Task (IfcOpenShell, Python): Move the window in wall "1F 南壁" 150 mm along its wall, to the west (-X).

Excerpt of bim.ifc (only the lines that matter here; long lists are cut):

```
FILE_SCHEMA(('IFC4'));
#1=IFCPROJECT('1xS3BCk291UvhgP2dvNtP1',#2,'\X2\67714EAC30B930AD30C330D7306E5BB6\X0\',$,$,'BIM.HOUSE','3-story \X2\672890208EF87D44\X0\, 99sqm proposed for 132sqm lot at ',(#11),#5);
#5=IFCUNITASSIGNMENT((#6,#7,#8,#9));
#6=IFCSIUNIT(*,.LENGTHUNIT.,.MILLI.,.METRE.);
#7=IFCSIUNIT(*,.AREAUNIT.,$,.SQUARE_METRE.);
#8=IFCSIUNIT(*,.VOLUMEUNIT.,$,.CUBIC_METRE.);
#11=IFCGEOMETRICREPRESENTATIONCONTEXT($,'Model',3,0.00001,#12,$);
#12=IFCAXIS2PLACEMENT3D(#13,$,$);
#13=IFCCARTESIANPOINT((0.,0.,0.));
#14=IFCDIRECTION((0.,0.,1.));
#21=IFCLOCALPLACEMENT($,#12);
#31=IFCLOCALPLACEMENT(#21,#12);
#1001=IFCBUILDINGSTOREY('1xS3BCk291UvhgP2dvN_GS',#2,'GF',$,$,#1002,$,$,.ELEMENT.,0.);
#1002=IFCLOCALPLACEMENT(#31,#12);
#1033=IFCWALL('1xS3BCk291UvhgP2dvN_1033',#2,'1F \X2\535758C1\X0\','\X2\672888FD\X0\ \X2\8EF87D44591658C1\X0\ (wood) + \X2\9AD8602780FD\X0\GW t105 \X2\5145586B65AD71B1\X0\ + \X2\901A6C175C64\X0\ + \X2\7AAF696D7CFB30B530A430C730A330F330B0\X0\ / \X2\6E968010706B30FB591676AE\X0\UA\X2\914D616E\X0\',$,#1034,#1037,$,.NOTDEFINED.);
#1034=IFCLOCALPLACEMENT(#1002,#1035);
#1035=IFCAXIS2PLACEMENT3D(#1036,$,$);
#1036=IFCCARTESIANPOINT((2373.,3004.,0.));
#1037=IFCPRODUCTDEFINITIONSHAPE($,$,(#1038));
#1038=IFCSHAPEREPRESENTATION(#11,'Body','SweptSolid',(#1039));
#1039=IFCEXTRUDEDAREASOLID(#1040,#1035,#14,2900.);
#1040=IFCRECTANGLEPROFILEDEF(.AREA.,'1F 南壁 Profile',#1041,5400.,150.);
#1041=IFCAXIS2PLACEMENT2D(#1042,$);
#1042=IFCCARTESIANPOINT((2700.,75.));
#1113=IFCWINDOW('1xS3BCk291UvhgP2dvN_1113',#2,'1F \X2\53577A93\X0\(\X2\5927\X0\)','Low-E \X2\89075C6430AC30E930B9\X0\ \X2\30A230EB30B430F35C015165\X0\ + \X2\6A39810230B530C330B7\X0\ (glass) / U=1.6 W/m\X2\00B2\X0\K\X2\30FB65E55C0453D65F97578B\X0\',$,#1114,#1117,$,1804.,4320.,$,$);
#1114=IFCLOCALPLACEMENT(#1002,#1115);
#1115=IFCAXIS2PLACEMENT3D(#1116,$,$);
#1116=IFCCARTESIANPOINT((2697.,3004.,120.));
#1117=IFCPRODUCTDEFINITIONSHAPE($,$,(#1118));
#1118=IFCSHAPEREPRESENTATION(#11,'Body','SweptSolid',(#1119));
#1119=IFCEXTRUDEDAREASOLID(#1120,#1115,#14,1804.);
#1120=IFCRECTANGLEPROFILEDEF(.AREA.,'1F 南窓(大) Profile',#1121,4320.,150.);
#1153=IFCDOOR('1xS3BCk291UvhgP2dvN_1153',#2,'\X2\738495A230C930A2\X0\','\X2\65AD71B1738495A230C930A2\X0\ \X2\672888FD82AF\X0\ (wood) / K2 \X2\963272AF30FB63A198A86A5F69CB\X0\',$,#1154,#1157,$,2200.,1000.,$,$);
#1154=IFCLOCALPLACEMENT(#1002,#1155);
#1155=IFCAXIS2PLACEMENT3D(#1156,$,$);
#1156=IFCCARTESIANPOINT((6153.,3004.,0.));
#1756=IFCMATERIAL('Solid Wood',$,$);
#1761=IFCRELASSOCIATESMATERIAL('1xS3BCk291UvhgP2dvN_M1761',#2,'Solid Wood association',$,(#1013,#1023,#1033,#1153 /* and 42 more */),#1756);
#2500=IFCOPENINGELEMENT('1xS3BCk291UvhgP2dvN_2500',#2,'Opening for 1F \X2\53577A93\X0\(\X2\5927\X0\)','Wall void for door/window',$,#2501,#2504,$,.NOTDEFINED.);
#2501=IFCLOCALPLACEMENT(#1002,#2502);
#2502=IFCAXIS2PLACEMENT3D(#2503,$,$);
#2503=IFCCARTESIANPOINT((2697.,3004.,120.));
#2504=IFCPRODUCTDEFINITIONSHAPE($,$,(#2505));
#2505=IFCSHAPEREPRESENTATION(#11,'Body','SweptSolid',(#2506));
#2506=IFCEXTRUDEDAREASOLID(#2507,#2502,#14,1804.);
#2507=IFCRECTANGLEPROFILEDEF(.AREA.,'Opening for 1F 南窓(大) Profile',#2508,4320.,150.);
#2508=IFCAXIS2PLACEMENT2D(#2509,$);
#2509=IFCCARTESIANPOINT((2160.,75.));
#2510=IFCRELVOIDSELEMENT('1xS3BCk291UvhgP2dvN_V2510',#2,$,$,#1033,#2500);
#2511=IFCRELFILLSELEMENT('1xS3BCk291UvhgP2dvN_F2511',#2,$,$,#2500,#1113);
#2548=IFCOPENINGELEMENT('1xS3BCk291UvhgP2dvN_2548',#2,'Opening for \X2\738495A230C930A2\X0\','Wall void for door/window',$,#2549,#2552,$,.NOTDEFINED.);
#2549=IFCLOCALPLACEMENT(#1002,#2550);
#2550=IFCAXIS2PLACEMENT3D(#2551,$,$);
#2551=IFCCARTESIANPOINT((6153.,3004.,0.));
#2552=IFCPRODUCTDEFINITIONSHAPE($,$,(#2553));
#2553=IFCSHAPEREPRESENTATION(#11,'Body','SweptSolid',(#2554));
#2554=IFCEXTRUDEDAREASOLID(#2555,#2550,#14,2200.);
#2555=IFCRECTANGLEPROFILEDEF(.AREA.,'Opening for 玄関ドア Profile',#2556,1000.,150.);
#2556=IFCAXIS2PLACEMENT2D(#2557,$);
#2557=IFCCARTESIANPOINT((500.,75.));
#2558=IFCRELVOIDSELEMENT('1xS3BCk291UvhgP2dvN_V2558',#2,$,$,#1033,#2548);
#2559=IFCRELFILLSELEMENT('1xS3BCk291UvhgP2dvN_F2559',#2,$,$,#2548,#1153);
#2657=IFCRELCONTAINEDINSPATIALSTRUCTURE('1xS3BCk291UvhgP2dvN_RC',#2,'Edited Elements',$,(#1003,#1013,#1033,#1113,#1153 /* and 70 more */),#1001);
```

```python
import ifcopenshell
import ifcopenshell.api.geometry
import ifcopenshell.util.placement

model = ifcopenshell.open("bim.ifc")

window = model.by_guid("1xS3BCk291UvhgP2dvN_1113")
opening = window.FillsVoids[0].RelatingOpeningElement
wall = opening.VoidsElements[0].RelatingBuildingElement

wall_matrix = ifcopenshell.util.placement.get_local_placement(wall.ObjectPlacement)
shift = wall_matrix[:3, 0] * -150.0
before = ifcopenshell.util.placement.get_local_placement(window.ObjectPlacement)[:3, 3].copy()

# The window is not placed relative to its opening, so move both.
for product in (opening, window):
    matrix = ifcopenshell.util.placement.get_local_placement(product.ObjectPlacement)
    matrix[:3, 3] += shift
    ifcopenshell.api.geometry.edit_object_placement(model, product=product, matrix=matrix, is_si=False)

after = ifcopenshell.util.placement.get_local_placement(window.ObjectPlacement)[:3, 3]
print("window moved by", (after - before).round(3) + 0.0)

model.write("bim_rev.ifc")
```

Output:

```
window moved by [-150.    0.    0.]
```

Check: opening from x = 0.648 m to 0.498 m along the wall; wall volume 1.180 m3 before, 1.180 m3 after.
